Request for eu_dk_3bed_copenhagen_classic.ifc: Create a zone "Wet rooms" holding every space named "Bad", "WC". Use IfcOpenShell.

First a look at what the model holds.

```python
import ifcopenshell

model = ifcopenshell.open("eu_dk_3bed_copenhagen_classic.ifc")
print(model.schema)
seen = {}
for space in model.by_type("IfcSpace"):
    seen[space.LongName] = seen.get(space.LongName, 0) + 1
for name, count in sorted(seen.items(), key=str):
    print(count, "x", name)
print("zones:", [z.Name for z in model.by_type("IfcZone")][:20])
```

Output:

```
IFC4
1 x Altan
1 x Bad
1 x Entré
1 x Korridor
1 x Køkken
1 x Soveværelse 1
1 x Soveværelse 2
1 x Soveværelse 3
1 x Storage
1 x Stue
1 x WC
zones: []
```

```python
import ifcopenshell
import ifcopenshell.api.group
import ifcopenshell.api.root

model = ifcopenshell.open("eu_dk_3bed_copenhagen_classic.ifc")

names = {"Bad", "WC"}
spaces = [s for s in model.by_type("IfcSpace") if s.LongName in names]

zone = ifcopenshell.api.root.create_entity(model, ifc_class="IfcZone", name="Wet rooms")
ifcopenshell.api.group.assign_group(model, products=spaces, group=zone)
print(len(spaces), "spaces in", zone.Name)

model.write("eu_dk_3bed_copenhagen_classic_v2.ifc")
```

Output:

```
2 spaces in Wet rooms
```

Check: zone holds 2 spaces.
